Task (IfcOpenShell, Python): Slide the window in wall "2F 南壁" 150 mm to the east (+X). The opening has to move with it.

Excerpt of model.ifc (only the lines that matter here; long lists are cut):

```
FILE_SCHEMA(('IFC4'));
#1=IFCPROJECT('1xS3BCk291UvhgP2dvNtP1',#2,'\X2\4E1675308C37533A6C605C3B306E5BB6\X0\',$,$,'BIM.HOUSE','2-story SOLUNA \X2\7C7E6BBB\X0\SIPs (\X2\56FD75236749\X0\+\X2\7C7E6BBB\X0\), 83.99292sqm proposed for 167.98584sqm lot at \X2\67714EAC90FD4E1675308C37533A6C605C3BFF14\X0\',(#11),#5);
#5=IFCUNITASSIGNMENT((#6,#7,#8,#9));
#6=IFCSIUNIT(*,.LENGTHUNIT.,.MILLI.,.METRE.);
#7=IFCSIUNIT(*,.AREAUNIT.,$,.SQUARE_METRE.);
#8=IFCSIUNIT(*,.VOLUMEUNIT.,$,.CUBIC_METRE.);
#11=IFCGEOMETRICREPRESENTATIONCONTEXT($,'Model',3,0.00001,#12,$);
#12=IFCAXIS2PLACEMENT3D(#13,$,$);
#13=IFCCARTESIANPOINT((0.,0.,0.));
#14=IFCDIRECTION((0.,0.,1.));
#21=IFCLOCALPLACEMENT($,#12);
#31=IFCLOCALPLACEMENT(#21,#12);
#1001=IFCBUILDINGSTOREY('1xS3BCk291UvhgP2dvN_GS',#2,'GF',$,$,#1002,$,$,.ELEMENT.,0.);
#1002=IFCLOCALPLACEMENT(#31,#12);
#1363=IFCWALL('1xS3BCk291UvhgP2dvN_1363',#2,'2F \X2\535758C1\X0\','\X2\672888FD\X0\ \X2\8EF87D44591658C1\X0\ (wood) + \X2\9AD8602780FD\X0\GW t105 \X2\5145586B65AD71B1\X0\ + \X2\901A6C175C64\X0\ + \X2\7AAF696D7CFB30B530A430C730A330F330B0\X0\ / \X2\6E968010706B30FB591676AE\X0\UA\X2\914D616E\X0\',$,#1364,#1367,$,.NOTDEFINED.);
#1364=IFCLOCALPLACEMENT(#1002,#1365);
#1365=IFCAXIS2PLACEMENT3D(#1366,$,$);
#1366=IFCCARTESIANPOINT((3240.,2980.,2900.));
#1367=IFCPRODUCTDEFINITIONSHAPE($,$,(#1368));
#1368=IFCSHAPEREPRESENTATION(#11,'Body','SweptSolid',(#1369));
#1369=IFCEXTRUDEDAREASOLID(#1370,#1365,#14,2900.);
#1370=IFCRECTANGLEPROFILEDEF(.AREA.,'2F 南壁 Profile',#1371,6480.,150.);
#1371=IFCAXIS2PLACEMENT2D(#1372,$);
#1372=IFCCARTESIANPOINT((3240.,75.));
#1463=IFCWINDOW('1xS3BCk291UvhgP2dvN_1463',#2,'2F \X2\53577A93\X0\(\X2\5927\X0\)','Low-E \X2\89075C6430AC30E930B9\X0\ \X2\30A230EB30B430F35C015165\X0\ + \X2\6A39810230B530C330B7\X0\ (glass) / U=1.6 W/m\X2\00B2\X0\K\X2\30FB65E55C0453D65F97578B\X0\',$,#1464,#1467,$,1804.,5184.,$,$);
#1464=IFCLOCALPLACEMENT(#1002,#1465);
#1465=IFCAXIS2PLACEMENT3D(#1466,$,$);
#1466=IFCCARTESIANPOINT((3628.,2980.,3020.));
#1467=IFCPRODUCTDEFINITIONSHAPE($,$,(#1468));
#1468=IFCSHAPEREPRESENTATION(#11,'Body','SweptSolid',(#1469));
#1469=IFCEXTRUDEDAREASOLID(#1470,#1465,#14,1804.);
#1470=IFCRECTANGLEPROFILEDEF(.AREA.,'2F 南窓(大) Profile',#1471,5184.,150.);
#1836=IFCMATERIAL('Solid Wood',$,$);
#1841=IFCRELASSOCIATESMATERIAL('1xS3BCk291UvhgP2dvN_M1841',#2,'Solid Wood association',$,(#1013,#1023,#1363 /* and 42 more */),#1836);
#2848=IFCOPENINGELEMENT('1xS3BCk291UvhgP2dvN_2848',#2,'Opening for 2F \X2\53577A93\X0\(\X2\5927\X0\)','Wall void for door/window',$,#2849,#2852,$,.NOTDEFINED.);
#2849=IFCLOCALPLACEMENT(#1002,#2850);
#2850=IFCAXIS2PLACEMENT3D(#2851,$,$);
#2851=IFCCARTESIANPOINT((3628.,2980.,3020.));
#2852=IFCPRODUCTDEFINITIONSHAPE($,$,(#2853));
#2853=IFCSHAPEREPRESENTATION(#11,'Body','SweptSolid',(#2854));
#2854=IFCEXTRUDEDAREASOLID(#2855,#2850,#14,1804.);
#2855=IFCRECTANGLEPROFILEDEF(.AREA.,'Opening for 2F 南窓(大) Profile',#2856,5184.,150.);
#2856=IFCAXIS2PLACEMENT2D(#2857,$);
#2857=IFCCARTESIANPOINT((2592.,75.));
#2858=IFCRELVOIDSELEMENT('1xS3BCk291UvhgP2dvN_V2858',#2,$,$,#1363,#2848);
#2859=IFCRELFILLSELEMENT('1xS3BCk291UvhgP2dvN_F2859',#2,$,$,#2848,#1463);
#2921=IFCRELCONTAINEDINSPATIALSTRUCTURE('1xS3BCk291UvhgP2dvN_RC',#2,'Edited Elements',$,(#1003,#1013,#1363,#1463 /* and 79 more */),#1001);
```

```python
import ifcopenshell
import ifcopenshell.api.geometry
import ifcopenshell.util.placement
import ifcopenshell.util.unit

model = ifcopenshell.open("model.ifc")
unit_scale = ifcopenshell.util.unit.calculate_unit_scale(model)

window = model.by_guid("1xS3BCk291UvhgP2dvN_1463")
opening = window.FillsVoids[0].RelatingOpeningElement
wall = opening.VoidsElements[0].RelatingBuildingElement

wall_matrix = ifcopenshell.util.placement.get_local_placement(wall.ObjectPlacement)
shift = wall_matrix[:3, 0] * 0.15 / unit_scale
before = ifcopenshell.util.placement.get_local_placement(window.ObjectPlacement)[:3, 3].copy()

# The window is not placed relative to its opening, so move both.
for product in (opening, window):
    matrix = ifcopenshell.util.placement.get_local_placement(product.ObjectPlacement)
    matrix[:3, 3] += shift
    ifcopenshell.api.geometry.edit_object_placement(model, product=product, matrix=matrix, is_si=False)

after = ifcopenshell.util.placement.get_local_placement(window.ObjectPlacement)[:3, 3]
print("window moved by", (after - before).round(3) + 0.0)

model.write("model_v2.ifc")
```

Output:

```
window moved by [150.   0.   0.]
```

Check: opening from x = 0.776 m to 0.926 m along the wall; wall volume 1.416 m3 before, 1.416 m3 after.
